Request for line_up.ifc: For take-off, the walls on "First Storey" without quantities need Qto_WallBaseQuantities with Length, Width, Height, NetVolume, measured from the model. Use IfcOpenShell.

First a look at what the model holds.

```python
import ifcopenshell
import ifcopenshell.util.element
import ifcopenshell.util.unit

model = ifcopenshell.open("line_up.ifc")
print(model.schema)
for unit_type in ("LENGTHUNIT", "AREAUNIT", "VOLUMEUNIT"):
    print(unit_type, ifcopenshell.util.unit.calculate_unit_scale(model, unit_type))
storey = next(s for s in model.by_type("IfcBuildingStorey") if s.Name == "First Storey")
walls = [e for e in ifcopenshell.util.element.get_decomposition(storey) if e.is_a("IfcWall")]
for e in sorted(walls, key=lambda e: e.id()):
    print(e.id(), e.is_a(), e.Name, list(ifcopenshell.util.element.get_psets(e, qtos_only=True)), sep=" | ")
```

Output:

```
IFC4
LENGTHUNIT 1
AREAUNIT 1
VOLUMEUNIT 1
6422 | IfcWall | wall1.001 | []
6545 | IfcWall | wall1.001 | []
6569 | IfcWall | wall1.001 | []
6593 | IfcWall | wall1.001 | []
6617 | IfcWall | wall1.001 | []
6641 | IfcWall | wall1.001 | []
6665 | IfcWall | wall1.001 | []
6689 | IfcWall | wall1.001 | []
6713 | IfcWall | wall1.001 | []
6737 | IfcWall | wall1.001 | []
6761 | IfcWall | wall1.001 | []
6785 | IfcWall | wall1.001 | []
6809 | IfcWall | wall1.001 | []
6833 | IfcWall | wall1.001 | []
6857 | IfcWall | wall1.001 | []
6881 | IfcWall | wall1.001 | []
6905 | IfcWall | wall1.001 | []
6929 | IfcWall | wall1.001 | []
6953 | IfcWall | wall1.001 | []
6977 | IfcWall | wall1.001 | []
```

```python
import ifcopenshell
import ifcopenshell.api.pset
import ifcopenshell.geom
import ifcopenshell.util.element
import ifcopenshell.util.shape
import ifcopenshell.util.unit

model = ifcopenshell.open("line_up.ifc")
unit_scale = ifcopenshell.util.unit.calculate_unit_scale(model)
volume_scale = ifcopenshell.util.unit.calculate_unit_scale(model, "VOLUMEUNIT")
settings = ifcopenshell.geom.settings()

storey = next(s for s in model.by_type("IfcBuildingStorey") if s.Name == "First Storey")
walls = [e for e in ifcopenshell.util.element.get_decomposition(storey) if e.is_a("IfcWall")]

for e in sorted(walls, key=lambda e: e.id()):
    if ifcopenshell.util.element.get_psets(e, qtos_only=True, should_inherit=False):
        continue
    # Geometry comes back in metres, in the element's own axes.
    shape = ifcopenshell.geom.create_shape(settings, e)
    values = {
        "Length": ifcopenshell.util.shape.get_x(shape.geometry) / unit_scale,
        "Width": ifcopenshell.util.shape.get_y(shape.geometry) / unit_scale,
        "Height": ifcopenshell.util.shape.get_z(shape.geometry) / unit_scale,
        "NetVolume": ifcopenshell.util.shape.get_volume(shape.geometry) / volume_scale,
    }
    qto = ifcopenshell.api.pset.add_qto(model, product=e, name="Qto_WallBaseQuantities")
    ifcopenshell.api.pset.edit_qto(model, qto=qto, properties=values)
    print(e.id(), {k: round(v, 3) for k, v in values.items()})

model.write("line_up_edited.ifc")
```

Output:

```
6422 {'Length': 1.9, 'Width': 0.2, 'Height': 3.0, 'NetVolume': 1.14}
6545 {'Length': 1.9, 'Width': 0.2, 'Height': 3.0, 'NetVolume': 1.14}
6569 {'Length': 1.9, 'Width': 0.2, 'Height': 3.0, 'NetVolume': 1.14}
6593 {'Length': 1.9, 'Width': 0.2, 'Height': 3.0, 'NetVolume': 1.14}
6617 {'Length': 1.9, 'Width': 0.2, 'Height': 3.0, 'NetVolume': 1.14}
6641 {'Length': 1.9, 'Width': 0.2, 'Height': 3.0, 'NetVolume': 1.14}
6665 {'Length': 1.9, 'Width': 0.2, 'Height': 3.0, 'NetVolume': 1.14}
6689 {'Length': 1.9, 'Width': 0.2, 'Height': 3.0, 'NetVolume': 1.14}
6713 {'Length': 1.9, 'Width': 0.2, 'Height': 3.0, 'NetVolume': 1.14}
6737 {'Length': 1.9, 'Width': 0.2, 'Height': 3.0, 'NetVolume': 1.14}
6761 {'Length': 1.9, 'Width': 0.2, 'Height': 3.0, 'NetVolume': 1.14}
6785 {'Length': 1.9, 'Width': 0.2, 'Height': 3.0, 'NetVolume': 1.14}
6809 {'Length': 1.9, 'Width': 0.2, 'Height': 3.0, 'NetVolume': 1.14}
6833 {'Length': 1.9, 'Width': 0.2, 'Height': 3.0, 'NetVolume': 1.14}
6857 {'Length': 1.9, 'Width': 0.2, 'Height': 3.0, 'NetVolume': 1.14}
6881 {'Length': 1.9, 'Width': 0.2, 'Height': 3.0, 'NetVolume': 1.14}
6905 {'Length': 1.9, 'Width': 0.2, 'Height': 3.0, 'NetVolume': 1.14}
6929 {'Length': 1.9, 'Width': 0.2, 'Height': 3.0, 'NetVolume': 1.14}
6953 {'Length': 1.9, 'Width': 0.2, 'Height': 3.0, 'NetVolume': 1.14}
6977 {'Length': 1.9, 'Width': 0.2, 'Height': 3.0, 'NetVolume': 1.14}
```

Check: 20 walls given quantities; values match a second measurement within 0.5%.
